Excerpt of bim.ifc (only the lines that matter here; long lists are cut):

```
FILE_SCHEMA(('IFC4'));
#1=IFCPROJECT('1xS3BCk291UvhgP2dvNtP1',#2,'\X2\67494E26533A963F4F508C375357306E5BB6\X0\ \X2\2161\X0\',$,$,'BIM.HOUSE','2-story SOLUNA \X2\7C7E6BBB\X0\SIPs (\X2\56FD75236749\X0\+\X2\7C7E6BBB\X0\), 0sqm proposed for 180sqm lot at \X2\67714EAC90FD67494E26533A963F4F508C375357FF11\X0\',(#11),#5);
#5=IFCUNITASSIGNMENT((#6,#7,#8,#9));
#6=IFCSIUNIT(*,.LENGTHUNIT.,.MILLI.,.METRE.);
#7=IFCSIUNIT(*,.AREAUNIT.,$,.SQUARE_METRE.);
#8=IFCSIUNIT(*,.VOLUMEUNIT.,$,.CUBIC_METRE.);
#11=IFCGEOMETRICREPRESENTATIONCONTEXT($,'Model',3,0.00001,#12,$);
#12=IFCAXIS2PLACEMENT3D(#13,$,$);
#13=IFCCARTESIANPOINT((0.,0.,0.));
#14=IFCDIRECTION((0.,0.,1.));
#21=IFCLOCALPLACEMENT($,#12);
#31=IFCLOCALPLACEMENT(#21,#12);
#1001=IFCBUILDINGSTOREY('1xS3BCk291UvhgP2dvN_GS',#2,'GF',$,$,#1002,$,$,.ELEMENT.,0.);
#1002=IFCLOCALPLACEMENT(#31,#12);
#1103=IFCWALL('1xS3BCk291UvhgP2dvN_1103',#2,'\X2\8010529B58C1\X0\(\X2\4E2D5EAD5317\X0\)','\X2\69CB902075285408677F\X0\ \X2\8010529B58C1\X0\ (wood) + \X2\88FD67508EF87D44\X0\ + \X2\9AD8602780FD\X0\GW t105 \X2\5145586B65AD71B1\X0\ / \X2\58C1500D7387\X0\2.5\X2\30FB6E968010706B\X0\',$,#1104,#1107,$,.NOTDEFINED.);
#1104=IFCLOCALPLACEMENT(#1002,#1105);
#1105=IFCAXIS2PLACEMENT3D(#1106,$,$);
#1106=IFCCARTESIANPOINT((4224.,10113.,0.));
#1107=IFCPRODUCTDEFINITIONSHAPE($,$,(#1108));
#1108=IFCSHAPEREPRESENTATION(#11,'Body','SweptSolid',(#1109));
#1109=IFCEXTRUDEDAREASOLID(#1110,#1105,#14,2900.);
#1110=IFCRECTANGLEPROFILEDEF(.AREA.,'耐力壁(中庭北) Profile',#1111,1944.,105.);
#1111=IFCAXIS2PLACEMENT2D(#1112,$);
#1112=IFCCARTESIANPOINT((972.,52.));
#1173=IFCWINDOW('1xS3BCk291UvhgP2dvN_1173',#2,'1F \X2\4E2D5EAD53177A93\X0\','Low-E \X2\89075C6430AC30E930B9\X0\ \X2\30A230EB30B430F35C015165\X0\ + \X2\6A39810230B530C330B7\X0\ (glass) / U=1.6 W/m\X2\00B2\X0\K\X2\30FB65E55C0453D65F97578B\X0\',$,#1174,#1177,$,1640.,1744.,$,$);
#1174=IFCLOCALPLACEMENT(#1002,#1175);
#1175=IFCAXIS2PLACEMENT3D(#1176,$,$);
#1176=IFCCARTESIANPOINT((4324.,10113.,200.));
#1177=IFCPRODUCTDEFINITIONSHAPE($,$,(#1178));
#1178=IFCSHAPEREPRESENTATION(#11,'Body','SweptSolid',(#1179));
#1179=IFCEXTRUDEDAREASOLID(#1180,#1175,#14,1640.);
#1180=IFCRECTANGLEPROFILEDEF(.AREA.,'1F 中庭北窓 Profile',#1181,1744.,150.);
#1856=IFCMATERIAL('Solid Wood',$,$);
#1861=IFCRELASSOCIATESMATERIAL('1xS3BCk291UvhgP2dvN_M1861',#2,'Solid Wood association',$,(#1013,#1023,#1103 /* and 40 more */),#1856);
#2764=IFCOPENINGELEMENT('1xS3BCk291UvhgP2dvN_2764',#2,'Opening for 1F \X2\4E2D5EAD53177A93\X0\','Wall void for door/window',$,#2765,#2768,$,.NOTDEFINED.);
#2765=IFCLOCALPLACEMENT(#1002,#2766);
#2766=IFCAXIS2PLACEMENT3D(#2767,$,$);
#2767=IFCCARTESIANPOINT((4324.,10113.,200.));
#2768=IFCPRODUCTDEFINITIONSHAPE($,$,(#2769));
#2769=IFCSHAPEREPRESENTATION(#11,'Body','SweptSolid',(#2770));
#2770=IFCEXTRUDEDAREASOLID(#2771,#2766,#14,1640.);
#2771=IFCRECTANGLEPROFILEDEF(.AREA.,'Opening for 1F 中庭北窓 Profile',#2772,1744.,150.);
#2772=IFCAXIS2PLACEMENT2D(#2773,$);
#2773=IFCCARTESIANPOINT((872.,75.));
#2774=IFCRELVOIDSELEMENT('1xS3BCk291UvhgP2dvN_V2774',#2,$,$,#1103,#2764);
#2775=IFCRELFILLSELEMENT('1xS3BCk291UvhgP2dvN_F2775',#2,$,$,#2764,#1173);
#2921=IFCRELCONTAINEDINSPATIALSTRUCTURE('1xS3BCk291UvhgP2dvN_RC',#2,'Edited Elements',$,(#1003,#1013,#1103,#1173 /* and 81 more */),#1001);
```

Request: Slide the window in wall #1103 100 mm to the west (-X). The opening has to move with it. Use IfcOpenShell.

```python
import ifcopenshell
import ifcopenshell.api.geometry
import ifcopenshell.util.placement
import ifcopenshell.util.unit

model = ifcopenshell.open("bim.ifc")
unit_scale = ifcopenshell.util.unit.calculate_unit_scale(model)

window = model.by_guid("1xS3BCk291UvhgP2dvN_1173")
opening = window.FillsVoids[0].RelatingOpeningElement
wall = opening.VoidsElements[0].RelatingBuildingElement

wall_matrix = ifcopenshell.util.placement.get_local_placement(wall.ObjectPlacement)
shift = wall_matrix[:3, 0] * -0.1 / unit_scale
before = ifcopenshell.util.placement.get_local_placement(window.ObjectPlacement)[:3, 3].copy()

# The window is not placed relative to its opening, so move both.
for product in (opening, window):
    matrix = ifcopenshell.util.placement.get_local_placement(product.ObjectPlacement)
    matrix[:3, 3] += shift
    ifcopenshell.api.geometry.edit_object_placement(model, product=product, matrix=matrix, is_si=False)

after = ifcopenshell.util.placement.get_local_placement(window.ObjectPlacement)[:3, 3]
print("window moved by", (after - before).round(3) + 0.0)

model.write("bim-out.ifc")
```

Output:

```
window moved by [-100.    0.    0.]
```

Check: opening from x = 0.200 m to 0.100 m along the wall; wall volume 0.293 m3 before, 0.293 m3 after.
